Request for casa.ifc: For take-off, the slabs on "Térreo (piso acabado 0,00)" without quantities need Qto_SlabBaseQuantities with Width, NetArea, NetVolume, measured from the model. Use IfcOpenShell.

First a look at what the model holds.

```python
import ifcopenshell
import ifcopenshell.util.element
import ifcopenshell.util.unit

model = ifcopenshell.open("casa.ifc")
print(model.schema)
for unit_type in ("LENGTHUNIT", "AREAUNIT", "VOLUMEUNIT"):
    print(unit_type, ifcopenshell.util.unit.calculate_unit_scale(model, unit_type))
storey = next(s for s in model.by_type("IfcBuildingStorey") if s.Name == "Térreo (piso acabado 0,00)")
slabs = [e for e in ifcopenshell.util.element.get_decomposition(storey) if e.is_a("IfcSlab")]
for e in sorted(slabs, key=lambda e: e.id()):
    print(e.id(), e.is_a(), e.Name, list(ifcopenshell.util.element.get_psets(e, qtos_only=True)), sep=" | ")
```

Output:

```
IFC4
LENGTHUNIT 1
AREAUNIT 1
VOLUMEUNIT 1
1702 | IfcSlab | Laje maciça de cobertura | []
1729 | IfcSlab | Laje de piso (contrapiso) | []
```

```python
import ifcopenshell
import ifcopenshell.api.pset
import ifcopenshell.geom
import ifcopenshell.util.element
import ifcopenshell.util.shape
import ifcopenshell.util.unit

model = ifcopenshell.open("casa.ifc")
unit_scale = ifcopenshell.util.unit.calculate_unit_scale(model)
area_scale = ifcopenshell.util.unit.calculate_unit_scale(model, "AREAUNIT")
volume_scale = ifcopenshell.util.unit.calculate_unit_scale(model, "VOLUMEUNIT")
settings = ifcopenshell.geom.settings()

storey = next(s for s in model.by_type("IfcBuildingStorey") if s.Name == "Térreo (piso acabado 0,00)")
slabs = [e for e in ifcopenshell.util.element.get_decomposition(storey) if e.is_a("IfcSlab")]

for e in sorted(slabs, key=lambda e: e.id()):
    if ifcopenshell.util.element.get_psets(e, qtos_only=True, should_inherit=False):
        continue
    # Geometry comes back in metres, in the element's own axes.
    shape = ifcopenshell.geom.create_shape(settings, e)
    values = {
        "Width": ifcopenshell.util.shape.get_z(shape.geometry) / unit_scale,
        "NetArea": ifcopenshell.util.shape.get_footprint_area(shape.geometry) / area_scale,
        "NetVolume": ifcopenshell.util.shape.get_volume(shape.geometry) / volume_scale,
    }
    qto = ifcopenshell.api.pset.add_qto(model, product=e, name="Qto_SlabBaseQuantities")
    ifcopenshell.api.pset.edit_qto(model, qto=qto, properties=values)
    print(e.id(), {k: round(v, 3) for k, v in values.items()})

model.write("casa_updated.ifc")
```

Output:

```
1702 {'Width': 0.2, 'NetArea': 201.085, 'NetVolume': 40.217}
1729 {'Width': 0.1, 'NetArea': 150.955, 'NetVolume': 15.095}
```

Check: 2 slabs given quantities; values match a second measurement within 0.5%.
